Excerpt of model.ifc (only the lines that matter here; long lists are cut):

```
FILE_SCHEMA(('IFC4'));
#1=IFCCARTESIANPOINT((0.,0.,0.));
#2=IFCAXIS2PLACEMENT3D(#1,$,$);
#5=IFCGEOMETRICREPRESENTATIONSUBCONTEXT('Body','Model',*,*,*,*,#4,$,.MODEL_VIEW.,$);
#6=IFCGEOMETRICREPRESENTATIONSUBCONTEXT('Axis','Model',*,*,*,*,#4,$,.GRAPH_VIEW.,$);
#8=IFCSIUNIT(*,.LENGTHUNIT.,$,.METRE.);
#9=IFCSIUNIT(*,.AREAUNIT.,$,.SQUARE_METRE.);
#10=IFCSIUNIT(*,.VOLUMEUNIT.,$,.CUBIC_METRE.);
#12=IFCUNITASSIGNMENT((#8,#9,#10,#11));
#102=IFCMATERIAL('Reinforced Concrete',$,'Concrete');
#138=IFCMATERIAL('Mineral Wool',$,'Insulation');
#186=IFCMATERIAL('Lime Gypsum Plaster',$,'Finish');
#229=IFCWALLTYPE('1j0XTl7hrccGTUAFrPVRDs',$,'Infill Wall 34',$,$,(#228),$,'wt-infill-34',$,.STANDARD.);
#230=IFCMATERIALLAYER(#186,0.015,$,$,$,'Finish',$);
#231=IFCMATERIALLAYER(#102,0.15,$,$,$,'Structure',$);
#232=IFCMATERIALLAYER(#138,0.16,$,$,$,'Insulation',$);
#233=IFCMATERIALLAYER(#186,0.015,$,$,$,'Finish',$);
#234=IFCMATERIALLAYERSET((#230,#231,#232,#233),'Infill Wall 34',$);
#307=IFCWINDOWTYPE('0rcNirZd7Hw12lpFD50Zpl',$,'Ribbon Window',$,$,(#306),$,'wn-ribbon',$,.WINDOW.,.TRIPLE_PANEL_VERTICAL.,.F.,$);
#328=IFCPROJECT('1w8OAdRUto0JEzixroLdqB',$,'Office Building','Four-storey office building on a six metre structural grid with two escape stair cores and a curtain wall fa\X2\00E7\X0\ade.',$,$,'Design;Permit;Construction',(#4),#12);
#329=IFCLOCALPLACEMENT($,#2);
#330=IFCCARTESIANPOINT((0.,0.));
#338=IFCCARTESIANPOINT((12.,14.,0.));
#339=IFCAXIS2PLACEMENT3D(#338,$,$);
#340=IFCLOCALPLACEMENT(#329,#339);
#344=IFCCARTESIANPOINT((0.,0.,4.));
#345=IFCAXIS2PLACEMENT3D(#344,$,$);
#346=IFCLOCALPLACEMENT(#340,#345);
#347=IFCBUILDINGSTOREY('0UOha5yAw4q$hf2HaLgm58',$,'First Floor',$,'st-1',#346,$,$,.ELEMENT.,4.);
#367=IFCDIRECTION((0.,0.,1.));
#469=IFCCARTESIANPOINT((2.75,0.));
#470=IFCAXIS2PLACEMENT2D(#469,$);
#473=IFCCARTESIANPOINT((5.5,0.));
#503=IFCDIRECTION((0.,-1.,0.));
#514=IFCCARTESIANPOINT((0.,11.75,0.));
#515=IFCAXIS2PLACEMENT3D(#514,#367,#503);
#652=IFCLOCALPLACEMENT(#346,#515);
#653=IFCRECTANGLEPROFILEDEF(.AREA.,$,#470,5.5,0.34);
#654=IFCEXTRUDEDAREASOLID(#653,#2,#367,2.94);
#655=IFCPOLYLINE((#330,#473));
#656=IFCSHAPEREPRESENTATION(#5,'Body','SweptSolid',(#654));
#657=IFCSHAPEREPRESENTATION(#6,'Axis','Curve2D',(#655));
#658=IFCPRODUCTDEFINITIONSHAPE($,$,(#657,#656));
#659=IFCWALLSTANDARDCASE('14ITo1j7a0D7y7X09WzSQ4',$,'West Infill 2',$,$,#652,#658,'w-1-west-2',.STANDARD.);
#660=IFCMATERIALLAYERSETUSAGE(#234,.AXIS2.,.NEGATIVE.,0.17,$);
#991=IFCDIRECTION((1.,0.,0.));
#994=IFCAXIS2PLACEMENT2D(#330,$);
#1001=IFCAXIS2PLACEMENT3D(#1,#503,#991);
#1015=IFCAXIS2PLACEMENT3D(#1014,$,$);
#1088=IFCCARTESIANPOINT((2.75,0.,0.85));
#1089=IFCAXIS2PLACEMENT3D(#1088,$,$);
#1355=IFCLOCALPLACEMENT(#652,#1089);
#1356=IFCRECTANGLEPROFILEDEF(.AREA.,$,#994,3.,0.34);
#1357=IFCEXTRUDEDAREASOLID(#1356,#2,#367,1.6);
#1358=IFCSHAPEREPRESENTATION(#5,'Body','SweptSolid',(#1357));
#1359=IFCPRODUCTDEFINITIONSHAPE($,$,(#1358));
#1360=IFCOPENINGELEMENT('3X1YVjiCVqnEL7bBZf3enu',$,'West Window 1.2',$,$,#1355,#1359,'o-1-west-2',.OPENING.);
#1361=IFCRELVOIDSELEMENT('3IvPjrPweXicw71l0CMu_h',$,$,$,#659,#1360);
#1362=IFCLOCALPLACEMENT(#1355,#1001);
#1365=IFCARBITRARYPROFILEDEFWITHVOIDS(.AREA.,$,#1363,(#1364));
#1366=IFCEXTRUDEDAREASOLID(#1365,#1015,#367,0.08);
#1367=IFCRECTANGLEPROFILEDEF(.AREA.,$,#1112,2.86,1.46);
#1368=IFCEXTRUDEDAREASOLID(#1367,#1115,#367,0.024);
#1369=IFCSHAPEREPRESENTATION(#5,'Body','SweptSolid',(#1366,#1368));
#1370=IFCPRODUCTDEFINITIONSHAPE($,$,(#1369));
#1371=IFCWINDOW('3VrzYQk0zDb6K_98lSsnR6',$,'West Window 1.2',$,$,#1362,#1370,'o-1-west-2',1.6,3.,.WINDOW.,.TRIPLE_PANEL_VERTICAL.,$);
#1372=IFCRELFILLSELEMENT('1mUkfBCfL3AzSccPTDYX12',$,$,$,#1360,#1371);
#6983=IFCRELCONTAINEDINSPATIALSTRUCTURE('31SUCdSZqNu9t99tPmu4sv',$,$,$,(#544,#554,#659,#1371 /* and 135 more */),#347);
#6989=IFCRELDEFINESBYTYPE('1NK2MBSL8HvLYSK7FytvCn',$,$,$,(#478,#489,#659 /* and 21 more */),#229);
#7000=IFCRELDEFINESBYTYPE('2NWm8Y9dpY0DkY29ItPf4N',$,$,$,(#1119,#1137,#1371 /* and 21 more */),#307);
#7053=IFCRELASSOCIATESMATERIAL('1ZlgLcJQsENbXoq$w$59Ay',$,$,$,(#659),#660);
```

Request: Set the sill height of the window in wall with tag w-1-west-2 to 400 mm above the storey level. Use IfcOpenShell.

```python
import numpy as np
import ifcopenshell
import ifcopenshell.api.geometry
import ifcopenshell.geom
import ifcopenshell.util.element
import ifcopenshell.util.placement
import ifcopenshell.util.shape
import ifcopenshell.util.unit

model = ifcopenshell.open("model.ifc")
unit_scale = ifcopenshell.util.unit.calculate_unit_scale(model)

window = model.by_guid("3VrzYQk0zDb6K_98lSsnR6")
opening = window.FillsVoids[0].RelatingOpeningElement
storey = ifcopenshell.util.element.get_container(window, ifc_class="IfcBuildingStorey")
level = ifcopenshell.util.placement.get_local_placement(storey.ObjectPlacement)[2, 3]

# The opening's origin need not be at the sill, so measure its lowest point.
shape = ifcopenshell.geom.create_shape(ifcopenshell.geom.settings(), opening)
bottom = ifcopenshell.util.shape.get_shape_bottom_elevation(shape, shape.geometry) / unit_scale
dz = level + 0.4 / unit_scale - bottom

shift = np.array([0.0, 0.0, dz])
# The window is placed relative to its opening, so it follows when the opening moves.
matrix = ifcopenshell.util.placement.get_local_placement(opening.ObjectPlacement)
matrix[:3, 3] += shift
ifcopenshell.api.geometry.edit_object_placement(
    model, product=opening, matrix=matrix, is_si=False, should_transform_children=True
)

print(f"moved by {dz * unit_scale:+.3f} m")

model.write("model_updated.ifc")
```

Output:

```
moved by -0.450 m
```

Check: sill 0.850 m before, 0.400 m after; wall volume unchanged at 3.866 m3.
